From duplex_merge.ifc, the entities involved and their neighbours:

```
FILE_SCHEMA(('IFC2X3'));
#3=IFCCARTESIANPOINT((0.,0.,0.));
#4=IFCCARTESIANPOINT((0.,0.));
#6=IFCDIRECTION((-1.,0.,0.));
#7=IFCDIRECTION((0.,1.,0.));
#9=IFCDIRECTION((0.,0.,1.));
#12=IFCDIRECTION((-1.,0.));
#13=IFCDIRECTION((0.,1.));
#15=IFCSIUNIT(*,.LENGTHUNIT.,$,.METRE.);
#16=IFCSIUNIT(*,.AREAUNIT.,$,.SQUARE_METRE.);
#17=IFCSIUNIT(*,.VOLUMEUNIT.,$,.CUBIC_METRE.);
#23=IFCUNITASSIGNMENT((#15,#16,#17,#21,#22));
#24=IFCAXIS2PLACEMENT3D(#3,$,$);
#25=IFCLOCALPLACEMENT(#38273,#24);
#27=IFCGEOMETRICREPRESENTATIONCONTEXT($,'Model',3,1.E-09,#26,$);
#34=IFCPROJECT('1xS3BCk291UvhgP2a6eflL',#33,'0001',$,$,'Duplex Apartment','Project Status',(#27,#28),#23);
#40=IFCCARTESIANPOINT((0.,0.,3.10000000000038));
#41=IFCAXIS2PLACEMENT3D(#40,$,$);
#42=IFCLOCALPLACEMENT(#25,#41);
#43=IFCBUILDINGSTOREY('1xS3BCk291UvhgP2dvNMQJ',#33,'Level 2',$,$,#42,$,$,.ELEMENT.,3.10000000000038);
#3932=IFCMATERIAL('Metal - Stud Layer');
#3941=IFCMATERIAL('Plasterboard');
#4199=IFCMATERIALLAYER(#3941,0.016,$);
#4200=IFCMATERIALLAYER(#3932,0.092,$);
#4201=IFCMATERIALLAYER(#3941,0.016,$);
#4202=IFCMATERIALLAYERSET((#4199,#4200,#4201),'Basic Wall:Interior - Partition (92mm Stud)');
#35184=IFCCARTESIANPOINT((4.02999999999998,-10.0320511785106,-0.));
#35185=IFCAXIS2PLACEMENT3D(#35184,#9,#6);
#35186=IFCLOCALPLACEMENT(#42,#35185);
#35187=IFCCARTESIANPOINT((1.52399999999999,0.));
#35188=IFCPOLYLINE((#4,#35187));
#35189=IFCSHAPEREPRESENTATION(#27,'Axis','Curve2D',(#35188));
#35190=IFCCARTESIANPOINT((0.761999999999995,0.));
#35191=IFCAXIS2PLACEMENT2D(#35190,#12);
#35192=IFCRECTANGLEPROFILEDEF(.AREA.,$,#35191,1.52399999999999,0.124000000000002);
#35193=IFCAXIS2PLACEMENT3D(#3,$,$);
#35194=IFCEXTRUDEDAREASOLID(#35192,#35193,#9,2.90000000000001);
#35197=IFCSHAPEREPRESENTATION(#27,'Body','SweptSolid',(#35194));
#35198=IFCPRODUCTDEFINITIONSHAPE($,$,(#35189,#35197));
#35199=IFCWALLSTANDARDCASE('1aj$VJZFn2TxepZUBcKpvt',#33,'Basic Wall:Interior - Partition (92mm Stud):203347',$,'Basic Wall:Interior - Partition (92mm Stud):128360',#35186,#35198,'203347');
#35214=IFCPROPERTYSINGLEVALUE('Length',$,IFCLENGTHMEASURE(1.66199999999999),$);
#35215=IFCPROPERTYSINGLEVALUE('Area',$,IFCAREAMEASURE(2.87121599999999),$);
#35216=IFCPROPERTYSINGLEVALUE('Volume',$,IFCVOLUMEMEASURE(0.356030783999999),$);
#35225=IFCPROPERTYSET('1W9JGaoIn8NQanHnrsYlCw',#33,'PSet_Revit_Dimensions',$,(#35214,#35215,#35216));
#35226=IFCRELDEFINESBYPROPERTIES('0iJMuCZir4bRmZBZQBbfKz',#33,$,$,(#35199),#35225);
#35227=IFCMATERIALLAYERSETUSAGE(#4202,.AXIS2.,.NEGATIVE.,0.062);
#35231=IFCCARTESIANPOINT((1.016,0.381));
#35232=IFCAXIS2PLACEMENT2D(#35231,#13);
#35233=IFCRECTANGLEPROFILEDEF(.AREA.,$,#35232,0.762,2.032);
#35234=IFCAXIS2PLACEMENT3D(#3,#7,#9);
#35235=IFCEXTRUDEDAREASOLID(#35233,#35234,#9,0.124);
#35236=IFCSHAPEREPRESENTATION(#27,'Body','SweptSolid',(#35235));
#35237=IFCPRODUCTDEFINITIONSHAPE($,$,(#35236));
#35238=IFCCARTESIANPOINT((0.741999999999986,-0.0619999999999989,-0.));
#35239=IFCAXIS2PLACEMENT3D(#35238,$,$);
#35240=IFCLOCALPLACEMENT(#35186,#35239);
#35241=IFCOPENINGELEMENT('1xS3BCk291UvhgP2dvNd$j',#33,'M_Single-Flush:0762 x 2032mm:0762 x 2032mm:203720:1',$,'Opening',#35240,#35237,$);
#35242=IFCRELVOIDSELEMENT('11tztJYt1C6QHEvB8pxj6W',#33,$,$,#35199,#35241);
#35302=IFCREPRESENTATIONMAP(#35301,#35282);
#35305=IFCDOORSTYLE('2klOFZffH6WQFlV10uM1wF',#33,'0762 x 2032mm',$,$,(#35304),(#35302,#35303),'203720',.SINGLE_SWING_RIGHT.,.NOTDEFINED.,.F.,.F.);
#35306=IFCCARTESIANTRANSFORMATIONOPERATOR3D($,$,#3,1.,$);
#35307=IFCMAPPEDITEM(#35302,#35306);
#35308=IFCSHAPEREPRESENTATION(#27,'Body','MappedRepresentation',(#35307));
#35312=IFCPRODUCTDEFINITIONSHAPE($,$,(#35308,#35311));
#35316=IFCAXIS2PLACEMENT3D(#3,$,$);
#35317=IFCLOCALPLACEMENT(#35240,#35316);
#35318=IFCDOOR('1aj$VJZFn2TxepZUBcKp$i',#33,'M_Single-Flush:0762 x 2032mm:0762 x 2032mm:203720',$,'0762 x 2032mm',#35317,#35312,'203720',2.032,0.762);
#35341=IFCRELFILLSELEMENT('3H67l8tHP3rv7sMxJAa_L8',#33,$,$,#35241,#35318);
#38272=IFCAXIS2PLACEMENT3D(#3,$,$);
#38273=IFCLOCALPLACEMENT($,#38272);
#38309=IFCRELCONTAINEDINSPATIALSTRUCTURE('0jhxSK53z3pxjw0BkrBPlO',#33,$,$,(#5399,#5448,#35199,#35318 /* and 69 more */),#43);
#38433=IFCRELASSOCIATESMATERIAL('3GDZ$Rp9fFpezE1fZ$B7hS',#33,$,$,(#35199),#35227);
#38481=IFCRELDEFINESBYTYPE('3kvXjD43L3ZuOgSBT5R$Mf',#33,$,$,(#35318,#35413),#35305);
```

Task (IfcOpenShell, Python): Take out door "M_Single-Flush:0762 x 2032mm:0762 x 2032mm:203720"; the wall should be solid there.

```python
import ifcopenshell
import ifcopenshell.api.feature
import ifcopenshell.api.pset
import ifcopenshell.api.root
import ifcopenshell.geom
import ifcopenshell.util.element
import ifcopenshell.util.shape
import ifcopenshell.util.unit

model = ifcopenshell.open("duplex_merge.ifc")
area_scale = ifcopenshell.util.unit.calculate_unit_scale(model, "AREAUNIT")
volume_scale = ifcopenshell.util.unit.calculate_unit_scale(model, "VOLUMEUNIT")
settings = ifcopenshell.geom.settings()


def volume(element):
    """Net volume in cubic metres, openings subtracted."""
    shape = ifcopenshell.geom.create_shape(settings, element)
    return ifcopenshell.util.shape.get_volume(shape.geometry)


door = model.by_guid("1aj$VJZFn2TxepZUBcKp$i")
opening = door.FillsVoids[0].RelatingOpeningElement
wall = opening.VoidsElements[0].RelatingBuildingElement
before = volume(wall)

ifcopenshell.api.root.remove_product(model, product=door)
ifcopenshell.api.feature.remove_feature(model, feature=opening)

after = volume(wall)
thickness = 0.124  # wall thickness in metres

# Update the wall's stored quantities.
pset = model.by_id(ifcopenshell.util.element.get_pset(wall, "PSet_Revit_Dimensions", should_inherit=False)["id"])
ifcopenshell.api.pset.edit_pset(model, pset=pset, properties={
    "Area": model.create_entity("IfcAreaMeasure", after / thickness / area_scale),
    "Volume": model.create_entity("IfcVolumeMeasure", after / volume_scale),
})

print(f"wall volume {before:.3f} -> {after:.3f} m3")

model.write("duplex_merge_edited.ifc")
```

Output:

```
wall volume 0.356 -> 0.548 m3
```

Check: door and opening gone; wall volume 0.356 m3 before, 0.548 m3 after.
